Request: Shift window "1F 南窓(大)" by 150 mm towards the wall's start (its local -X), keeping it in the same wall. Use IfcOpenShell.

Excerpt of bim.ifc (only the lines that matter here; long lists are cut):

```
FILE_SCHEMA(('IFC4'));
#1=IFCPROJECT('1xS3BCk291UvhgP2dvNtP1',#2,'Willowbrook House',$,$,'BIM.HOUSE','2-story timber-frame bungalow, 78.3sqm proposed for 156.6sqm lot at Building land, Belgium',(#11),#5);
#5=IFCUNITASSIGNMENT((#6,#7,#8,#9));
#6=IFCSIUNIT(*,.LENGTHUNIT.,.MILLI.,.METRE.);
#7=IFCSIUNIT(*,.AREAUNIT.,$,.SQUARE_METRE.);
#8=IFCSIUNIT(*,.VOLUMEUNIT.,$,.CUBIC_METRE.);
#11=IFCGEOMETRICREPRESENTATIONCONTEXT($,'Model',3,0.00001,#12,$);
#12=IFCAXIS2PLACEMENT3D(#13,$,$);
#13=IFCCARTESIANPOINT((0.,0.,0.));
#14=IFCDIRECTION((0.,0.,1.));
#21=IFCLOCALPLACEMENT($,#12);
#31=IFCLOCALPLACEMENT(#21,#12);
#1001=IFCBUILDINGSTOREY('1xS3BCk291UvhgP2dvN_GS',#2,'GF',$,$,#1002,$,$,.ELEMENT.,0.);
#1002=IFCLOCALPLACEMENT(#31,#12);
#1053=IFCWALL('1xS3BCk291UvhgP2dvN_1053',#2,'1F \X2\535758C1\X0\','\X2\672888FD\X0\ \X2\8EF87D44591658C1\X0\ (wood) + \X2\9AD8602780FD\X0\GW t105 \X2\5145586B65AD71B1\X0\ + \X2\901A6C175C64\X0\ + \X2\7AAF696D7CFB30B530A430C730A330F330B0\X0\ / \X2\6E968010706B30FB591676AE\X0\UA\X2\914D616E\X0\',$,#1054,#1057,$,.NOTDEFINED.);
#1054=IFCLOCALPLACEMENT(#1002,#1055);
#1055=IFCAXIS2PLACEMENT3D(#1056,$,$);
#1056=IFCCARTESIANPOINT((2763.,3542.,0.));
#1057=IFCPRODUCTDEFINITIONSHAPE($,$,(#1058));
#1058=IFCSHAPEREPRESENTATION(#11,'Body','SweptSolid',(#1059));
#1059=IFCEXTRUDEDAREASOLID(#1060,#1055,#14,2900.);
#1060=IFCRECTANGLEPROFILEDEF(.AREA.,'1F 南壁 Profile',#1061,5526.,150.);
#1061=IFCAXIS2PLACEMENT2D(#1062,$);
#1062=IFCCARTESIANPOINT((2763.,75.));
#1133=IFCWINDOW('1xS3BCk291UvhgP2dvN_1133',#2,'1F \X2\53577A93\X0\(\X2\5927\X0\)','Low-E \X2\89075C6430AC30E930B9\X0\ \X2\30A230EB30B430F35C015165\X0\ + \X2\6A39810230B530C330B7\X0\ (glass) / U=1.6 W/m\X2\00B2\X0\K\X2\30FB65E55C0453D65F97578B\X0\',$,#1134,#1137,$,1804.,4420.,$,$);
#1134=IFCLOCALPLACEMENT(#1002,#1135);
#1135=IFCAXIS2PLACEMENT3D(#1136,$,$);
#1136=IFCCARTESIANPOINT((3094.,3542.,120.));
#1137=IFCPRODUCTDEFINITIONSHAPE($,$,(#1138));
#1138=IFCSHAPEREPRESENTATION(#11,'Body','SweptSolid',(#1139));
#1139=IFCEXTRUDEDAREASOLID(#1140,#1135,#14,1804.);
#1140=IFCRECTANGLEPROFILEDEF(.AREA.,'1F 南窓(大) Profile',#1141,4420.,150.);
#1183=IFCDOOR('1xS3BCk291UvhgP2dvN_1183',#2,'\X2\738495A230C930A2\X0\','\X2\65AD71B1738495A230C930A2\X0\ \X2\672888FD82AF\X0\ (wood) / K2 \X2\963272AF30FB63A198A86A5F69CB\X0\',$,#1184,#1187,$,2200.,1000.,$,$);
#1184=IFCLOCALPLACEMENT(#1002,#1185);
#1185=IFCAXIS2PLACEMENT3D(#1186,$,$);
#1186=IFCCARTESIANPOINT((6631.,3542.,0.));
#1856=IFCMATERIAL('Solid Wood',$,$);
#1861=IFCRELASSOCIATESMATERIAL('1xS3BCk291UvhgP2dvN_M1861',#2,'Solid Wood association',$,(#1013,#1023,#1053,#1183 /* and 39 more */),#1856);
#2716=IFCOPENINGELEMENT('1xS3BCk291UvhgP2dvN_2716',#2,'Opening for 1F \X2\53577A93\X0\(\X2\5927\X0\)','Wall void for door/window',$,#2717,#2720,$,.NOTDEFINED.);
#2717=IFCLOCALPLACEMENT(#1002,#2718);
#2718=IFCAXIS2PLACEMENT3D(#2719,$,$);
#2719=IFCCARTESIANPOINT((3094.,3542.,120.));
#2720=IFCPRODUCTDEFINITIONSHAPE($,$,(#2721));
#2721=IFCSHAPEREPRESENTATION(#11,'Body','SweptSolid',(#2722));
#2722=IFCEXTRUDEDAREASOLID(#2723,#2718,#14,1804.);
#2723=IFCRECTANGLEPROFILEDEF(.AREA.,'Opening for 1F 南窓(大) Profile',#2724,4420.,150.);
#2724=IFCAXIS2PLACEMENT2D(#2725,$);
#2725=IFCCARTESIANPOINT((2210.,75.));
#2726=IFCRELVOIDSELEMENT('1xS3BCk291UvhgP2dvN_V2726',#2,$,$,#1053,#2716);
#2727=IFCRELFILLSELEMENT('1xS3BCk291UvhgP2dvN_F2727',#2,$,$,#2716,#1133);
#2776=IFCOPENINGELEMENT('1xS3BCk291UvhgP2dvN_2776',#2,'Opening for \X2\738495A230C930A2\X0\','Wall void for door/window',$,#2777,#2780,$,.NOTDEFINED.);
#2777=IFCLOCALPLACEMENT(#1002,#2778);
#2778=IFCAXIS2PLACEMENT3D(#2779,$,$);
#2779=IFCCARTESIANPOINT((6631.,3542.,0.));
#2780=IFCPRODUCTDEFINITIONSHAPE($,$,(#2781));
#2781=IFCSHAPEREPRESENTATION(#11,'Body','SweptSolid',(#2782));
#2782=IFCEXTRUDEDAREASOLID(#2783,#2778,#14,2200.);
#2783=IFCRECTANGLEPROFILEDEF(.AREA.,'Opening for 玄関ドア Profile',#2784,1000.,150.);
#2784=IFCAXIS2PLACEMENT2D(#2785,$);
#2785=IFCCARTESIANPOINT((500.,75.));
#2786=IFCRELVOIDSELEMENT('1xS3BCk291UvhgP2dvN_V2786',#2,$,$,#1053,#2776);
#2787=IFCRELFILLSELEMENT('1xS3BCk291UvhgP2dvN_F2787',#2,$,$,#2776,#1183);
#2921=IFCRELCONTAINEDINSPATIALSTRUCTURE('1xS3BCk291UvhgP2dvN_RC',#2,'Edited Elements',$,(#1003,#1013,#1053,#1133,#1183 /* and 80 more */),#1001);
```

```python
import ifcopenshell
import ifcopenshell.api.geometry
import ifcopenshell.util.placement

model = ifcopenshell.open("bim.ifc")

window = model.by_guid("1xS3BCk291UvhgP2dvN_1133")
opening = window.FillsVoids[0].RelatingOpeningElement
wall = opening.VoidsElements[0].RelatingBuildingElement

wall_matrix = ifcopenshell.util.placement.get_local_placement(wall.ObjectPlacement)
shift = wall_matrix[:3, 0] * -150.0
before = ifcopenshell.util.placement.get_local_placement(window.ObjectPlacement)[:3, 3].copy()

# The window is not placed relative to its opening, so move both.
for product in (opening, window):
    matrix = ifcopenshell.util.placement.get_local_placement(product.ObjectPlacement)
    matrix[:3, 3] += shift
    ifcopenshell.api.geometry.edit_object_placement(model, product=product, matrix=matrix, is_si=False)

after = ifcopenshell.util.placement.get_local_placement(window.ObjectPlacement)[:3, 3]
print("window moved by", (after - before).round(3) + 0.0)

model.write("bim-out.ifc")
```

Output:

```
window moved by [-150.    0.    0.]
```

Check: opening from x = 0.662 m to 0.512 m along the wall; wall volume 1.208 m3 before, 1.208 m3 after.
